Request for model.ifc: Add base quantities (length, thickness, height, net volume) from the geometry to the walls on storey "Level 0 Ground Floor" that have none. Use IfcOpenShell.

First a look at what the model holds.

```python
import ifcopenshell
import ifcopenshell.util.element
import ifcopenshell.util.unit

model = ifcopenshell.open("model.ifc")
print(model.schema)
for unit_type in ("LENGTHUNIT", "AREAUNIT", "VOLUMEUNIT"):
    print(unit_type, ifcopenshell.util.unit.calculate_unit_scale(model, unit_type))
storey = next(s for s in model.by_type("IfcBuildingStorey") if s.Name == "Level 0 Ground Floor")
walls = [e for e in ifcopenshell.util.element.get_decomposition(storey) if e.is_a("IfcWall")]
for e in sorted(walls, key=lambda e: e.id()):
    print(e.id(), e.is_a(), e.Name, list(ifcopenshell.util.element.get_psets(e, qtos_only=True)), sep=" | ")
```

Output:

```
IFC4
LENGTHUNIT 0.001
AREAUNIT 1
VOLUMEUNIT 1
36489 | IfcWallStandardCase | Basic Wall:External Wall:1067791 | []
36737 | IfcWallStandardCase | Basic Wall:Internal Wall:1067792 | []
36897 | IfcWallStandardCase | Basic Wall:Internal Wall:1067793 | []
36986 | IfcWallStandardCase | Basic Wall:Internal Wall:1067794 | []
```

```python
import ifcopenshell
import ifcopenshell.api.pset
import ifcopenshell.geom
import ifcopenshell.util.element
import ifcopenshell.util.shape
import ifcopenshell.util.unit

model = ifcopenshell.open("model.ifc")
unit_scale = ifcopenshell.util.unit.calculate_unit_scale(model)
volume_scale = ifcopenshell.util.unit.calculate_unit_scale(model, "VOLUMEUNIT")
settings = ifcopenshell.geom.settings()

storey = next(s for s in model.by_type("IfcBuildingStorey") if s.Name == "Level 0 Ground Floor")
walls = [e for e in ifcopenshell.util.element.get_decomposition(storey) if e.is_a("IfcWall")]

for e in sorted(walls, key=lambda e: e.id()):
    if ifcopenshell.util.element.get_psets(e, qtos_only=True, should_inherit=False):
        continue
    # Geometry comes back in metres, in the element's own axes.
    shape = ifcopenshell.geom.create_shape(settings, e)
    values = {
        "Length": ifcopenshell.util.shape.get_x(shape.geometry) / unit_scale,
        "Width": ifcopenshell.util.shape.get_y(shape.geometry) / unit_scale,
        "Height": ifcopenshell.util.shape.get_z(shape.geometry) / unit_scale,
        "NetVolume": ifcopenshell.util.shape.get_volume(shape.geometry) / volume_scale,
    }
    qto = ifcopenshell.api.pset.add_qto(model, product=e, name="Qto_WallBaseQuantities")
    ifcopenshell.api.pset.edit_qto(model, qto=qto, properties=values)
    print(e.id(), {k: round(v, 3) for k, v in values.items()})

model.write("model_v2.ifc")
```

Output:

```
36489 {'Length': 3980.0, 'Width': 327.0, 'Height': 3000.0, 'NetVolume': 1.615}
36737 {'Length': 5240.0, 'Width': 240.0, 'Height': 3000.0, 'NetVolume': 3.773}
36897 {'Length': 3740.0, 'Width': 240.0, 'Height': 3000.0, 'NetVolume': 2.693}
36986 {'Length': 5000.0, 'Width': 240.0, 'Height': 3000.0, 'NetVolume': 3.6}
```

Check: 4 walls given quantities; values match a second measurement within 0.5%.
